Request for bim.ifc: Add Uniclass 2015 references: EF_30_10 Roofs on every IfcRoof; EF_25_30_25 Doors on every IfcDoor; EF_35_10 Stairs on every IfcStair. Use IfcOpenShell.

First a look at what the model holds.

```python
import ifcopenshell

model = ifcopenshell.open("bim.ifc")
print(model.schema)
print("classifications:", [c.Name for c in model.by_type("IfcClassification")])
for ifc_class in ("IfcDoor", "IfcRoof", "IfcStair", "IfcWall", "IfcWindow"):
    print(ifc_class, len(model.by_type(ifc_class)))
```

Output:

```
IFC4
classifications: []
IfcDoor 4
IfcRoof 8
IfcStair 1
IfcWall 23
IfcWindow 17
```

```python
import ifcopenshell
import ifcopenshell.api.classification

model = ifcopenshell.open("bim.ifc")

system = ifcopenshell.api.classification.add_classification(model, classification="Uniclass 2015")

codes = {
    "IfcRoof": ("EF_30_10", "Roofs"),
    "IfcDoor": ("EF_25_30_25", "Doors"),
    "IfcStair": ("EF_35_10", "Stairs"),
}
for ifc_class, (code, name) in codes.items():
    products = model.by_type(ifc_class)
    ifcopenshell.api.classification.add_reference(
        model, products=products, classification=system, identification=code, name=name
    )
    print(code, len(products))

model.write("bim_v2.ifc")
```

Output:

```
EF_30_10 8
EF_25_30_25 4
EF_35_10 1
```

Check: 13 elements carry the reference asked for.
